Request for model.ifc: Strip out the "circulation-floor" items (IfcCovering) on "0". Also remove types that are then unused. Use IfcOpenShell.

First a look at what the model holds.

```python
import ifcopenshell
import ifcopenshell.util.element

model = ifcopenshell.open("model.ifc")
print(model.schema)
storey = next(s for s in model.by_type("IfcBuildingStorey") if s.Name == "0")
coverings = [e for e in ifcopenshell.util.element.get_decomposition(storey) if e.is_a("IfcCovering")]
seen = {}
for e in coverings:
    element_type = ifcopenshell.util.element.get_type(e)
    name = element_type.Name if element_type not in (None, e) else None
    seen[name] = seen.get(name, 0) + 1
for name, count in sorted(seen.items(), key=str):
    print(count, "x", name)
```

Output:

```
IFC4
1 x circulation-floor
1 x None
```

```python
import ifcopenshell
import ifcopenshell.api.root
import ifcopenshell.util.element

model = ifcopenshell.open("model.ifc")

storey = next(s for s in model.by_type("IfcBuildingStorey") if s.Name == "0")
coverings = [e for e in ifcopenshell.util.element.get_decomposition(storey) if e.is_a("IfcCovering")]
targets = [e for e in coverings if (t := ifcopenshell.util.element.get_type(e)) not in (None, e) and t.Name == "circulation-floor"]
types = {ifcopenshell.util.element.get_type(e) for e in targets} - {None, *targets}

for e in targets:
    ifcopenshell.api.root.remove_product(model, product=e)
print(len(targets), "removed")

unused = [t for t in types if not ifcopenshell.util.element.get_types(t)]
for t in unused:
    ifcopenshell.api.root.remove_product(model, product=t)
print(len(unused), "unused types removed")

model.write("model-out.ifc")
```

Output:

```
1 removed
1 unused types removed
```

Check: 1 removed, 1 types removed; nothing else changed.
